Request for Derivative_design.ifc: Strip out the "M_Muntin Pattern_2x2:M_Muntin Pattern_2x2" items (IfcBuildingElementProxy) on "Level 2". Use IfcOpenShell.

First a look at what the model holds.

```python
import ifcopenshell
import ifcopenshell.util.element

model = ifcopenshell.open("Derivative_design.ifc")
print(model.schema)
storey = next(s for s in model.by_type("IfcBuildingStorey") if s.Name == "Level 2")
proxies = [e for e in ifcopenshell.util.element.get_decomposition(storey) if e.is_a("IfcBuildingElementProxy")]
seen = {}
for e in proxies:
    element_type = ifcopenshell.util.element.get_type(e)
    name = element_type.Name if element_type not in (None, e) else None
    seen[name] = seen.get(name, 0) + 1
for name, count in sorted(seen.items(), key=str):
    print(count, "x", name)
```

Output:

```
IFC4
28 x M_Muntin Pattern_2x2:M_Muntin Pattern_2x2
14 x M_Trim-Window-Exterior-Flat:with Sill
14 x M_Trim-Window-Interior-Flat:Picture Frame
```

```python
import ifcopenshell
import ifcopenshell.api.root
import ifcopenshell.util.element

model = ifcopenshell.open("Derivative_design.ifc")

storey = next(s for s in model.by_type("IfcBuildingStorey") if s.Name == "Level 2")
proxies = [e for e in ifcopenshell.util.element.get_decomposition(storey) if e.is_a("IfcBuildingElementProxy")]
targets = [e for e in proxies if (t := ifcopenshell.util.element.get_type(e)) not in (None, e) and t.Name == "M_Muntin Pattern_2x2:M_Muntin Pattern_2x2"]

for e in targets:
    ifcopenshell.api.root.remove_product(model, product=e)
print(len(targets), "removed")

model.write("Derivative_design_v2.ifc")
```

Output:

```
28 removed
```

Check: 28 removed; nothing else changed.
